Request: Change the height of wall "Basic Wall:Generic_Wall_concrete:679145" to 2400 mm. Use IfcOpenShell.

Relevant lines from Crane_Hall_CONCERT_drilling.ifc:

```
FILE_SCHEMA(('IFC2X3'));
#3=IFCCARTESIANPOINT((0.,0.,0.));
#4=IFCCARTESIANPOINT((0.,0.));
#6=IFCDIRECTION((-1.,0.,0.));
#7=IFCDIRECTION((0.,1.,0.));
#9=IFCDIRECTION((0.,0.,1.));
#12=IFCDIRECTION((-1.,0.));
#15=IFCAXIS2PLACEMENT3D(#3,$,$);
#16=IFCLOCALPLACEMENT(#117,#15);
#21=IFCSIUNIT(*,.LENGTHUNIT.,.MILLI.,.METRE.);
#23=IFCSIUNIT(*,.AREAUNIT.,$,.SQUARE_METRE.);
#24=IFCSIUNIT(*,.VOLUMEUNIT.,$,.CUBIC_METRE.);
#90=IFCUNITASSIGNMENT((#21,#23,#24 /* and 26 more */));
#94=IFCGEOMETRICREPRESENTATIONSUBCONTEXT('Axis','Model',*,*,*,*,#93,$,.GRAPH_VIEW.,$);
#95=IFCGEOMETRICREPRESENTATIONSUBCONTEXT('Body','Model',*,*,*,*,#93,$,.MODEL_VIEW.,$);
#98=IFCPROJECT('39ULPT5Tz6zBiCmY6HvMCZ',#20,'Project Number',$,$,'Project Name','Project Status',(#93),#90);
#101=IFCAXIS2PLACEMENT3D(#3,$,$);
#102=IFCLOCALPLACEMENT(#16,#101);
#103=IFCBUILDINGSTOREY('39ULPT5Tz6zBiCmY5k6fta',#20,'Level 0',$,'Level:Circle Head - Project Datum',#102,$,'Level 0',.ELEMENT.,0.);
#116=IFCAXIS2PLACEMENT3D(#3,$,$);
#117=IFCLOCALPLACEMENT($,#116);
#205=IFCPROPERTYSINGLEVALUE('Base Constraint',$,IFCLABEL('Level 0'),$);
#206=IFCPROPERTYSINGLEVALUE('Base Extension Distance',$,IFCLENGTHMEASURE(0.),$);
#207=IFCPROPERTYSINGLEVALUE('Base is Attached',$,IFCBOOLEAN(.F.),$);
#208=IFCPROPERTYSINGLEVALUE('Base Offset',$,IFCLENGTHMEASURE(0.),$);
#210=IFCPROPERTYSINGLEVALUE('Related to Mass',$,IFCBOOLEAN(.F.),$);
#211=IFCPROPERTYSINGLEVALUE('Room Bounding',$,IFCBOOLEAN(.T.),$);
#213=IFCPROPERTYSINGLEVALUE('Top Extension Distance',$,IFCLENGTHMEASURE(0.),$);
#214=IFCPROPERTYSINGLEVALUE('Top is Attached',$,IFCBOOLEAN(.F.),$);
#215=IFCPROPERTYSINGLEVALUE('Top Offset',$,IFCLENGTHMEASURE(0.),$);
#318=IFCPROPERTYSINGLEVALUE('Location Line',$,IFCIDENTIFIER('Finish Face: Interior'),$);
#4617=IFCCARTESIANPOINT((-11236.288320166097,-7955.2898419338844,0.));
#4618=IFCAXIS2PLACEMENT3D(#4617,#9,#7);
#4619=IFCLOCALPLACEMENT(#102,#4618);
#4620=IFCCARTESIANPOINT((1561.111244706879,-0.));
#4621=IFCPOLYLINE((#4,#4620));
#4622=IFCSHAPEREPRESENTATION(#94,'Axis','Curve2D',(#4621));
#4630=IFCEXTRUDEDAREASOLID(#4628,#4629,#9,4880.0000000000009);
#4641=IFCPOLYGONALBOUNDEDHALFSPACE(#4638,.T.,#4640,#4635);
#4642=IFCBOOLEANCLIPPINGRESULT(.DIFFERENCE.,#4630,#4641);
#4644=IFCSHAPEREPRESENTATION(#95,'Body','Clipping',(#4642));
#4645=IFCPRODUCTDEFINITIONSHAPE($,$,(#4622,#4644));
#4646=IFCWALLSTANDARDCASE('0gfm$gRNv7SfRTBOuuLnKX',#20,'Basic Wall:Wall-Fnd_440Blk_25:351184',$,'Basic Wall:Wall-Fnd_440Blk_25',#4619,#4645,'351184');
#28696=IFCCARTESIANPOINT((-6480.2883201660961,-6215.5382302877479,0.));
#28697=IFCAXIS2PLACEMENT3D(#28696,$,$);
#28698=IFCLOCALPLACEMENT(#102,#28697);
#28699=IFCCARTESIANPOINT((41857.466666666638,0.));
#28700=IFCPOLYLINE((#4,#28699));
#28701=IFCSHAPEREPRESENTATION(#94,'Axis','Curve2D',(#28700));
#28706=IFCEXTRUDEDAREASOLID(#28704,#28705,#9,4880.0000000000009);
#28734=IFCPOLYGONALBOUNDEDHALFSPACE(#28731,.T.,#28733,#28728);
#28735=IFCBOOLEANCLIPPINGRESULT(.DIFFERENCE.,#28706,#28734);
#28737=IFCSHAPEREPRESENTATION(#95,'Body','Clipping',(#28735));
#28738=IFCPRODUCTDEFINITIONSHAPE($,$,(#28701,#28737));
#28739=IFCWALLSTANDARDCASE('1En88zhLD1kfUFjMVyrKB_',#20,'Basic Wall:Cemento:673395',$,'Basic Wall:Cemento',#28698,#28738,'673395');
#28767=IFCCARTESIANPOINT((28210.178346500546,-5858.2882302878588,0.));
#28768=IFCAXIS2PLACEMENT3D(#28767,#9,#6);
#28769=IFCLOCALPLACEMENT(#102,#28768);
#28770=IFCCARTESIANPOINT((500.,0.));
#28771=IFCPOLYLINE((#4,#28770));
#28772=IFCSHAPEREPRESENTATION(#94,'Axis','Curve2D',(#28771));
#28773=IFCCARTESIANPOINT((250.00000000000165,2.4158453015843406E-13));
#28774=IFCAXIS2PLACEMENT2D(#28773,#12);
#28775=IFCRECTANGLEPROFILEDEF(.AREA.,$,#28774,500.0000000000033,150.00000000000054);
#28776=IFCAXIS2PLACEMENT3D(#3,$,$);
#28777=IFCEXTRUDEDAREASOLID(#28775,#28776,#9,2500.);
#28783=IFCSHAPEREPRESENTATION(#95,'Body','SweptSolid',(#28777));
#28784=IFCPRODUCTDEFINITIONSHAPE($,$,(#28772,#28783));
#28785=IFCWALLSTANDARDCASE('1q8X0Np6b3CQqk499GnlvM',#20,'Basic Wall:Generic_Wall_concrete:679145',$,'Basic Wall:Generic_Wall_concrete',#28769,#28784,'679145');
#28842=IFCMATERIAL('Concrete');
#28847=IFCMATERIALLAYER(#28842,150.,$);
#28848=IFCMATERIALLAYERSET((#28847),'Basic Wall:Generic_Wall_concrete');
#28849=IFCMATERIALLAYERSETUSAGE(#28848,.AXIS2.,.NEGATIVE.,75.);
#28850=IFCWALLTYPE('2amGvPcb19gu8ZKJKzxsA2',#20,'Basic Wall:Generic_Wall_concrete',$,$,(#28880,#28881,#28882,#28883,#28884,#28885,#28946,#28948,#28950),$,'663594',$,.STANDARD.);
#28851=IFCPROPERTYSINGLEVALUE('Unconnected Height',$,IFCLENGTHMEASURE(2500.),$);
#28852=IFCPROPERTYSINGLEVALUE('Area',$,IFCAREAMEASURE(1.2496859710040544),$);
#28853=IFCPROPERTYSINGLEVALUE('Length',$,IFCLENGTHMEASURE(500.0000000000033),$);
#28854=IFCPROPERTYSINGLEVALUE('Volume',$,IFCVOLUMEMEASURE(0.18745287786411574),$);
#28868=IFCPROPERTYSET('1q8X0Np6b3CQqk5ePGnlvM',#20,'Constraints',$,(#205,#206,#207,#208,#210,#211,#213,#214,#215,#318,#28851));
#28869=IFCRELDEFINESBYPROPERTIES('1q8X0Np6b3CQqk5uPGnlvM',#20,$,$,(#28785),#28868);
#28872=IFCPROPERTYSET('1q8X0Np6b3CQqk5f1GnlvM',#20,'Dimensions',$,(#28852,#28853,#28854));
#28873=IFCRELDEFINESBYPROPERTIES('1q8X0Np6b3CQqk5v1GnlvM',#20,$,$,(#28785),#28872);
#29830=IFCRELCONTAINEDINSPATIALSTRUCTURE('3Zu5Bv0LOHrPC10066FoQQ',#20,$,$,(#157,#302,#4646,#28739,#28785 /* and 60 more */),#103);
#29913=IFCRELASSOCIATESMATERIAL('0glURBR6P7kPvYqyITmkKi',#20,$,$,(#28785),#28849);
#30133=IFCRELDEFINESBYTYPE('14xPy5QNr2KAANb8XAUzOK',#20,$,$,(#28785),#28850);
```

```python
import ifcopenshell
import ifcopenshell.api.pset
import ifcopenshell.geom
import ifcopenshell.util.element
import ifcopenshell.util.representation
import ifcopenshell.util.shape
import ifcopenshell.util.unit

model = ifcopenshell.open("Crane_Hall_CONCERT_drilling.ifc")
unit_scale = ifcopenshell.util.unit.calculate_unit_scale(model)
area_scale = ifcopenshell.util.unit.calculate_unit_scale(model, "AREAUNIT")
volume_scale = ifcopenshell.util.unit.calculate_unit_scale(model, "VOLUMEUNIT")
settings = ifcopenshell.geom.settings()


def volume(element):
    """Net volume in cubic metres, openings subtracted."""
    shape = ifcopenshell.geom.create_shape(settings, element)
    return ifcopenshell.util.shape.get_volume(shape.geometry)


wall = model.by_id(28785)
before = volume(wall)

body = ifcopenshell.util.representation.get_representation(wall, "Model", "Body")
solid = body.Items[0]
old_height = solid.Depth
solid.Depth = 2.4 / unit_scale
after = volume(wall)
thickness = 0.15  # wall thickness in metres

# Update the stored height, areas and volumes.
pset = model.by_id(ifcopenshell.util.element.get_pset(wall, "Constraints", should_inherit=False)["id"])
ifcopenshell.api.pset.edit_pset(model, pset=pset, properties={
    "Unconnected Height": model.create_entity("IfcLengthMeasure", solid.Depth),
})
pset = model.by_id(ifcopenshell.util.element.get_pset(wall, "Dimensions", should_inherit=False)["id"])
ifcopenshell.api.pset.edit_pset(model, pset=pset, properties={
    "Area": model.create_entity("IfcAreaMeasure", after / thickness / area_scale),
    "Volume": model.create_entity("IfcVolumeMeasure", after / volume_scale),
})

print(f"height {old_height:g} -> {solid.Depth:g}, volume {before:.3f} -> {after:.3f} m3")

model.write("Crane_Hall_CONCERT_drilling-out.ifc")
```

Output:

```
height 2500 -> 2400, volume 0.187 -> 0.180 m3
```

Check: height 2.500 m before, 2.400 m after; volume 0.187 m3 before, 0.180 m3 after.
